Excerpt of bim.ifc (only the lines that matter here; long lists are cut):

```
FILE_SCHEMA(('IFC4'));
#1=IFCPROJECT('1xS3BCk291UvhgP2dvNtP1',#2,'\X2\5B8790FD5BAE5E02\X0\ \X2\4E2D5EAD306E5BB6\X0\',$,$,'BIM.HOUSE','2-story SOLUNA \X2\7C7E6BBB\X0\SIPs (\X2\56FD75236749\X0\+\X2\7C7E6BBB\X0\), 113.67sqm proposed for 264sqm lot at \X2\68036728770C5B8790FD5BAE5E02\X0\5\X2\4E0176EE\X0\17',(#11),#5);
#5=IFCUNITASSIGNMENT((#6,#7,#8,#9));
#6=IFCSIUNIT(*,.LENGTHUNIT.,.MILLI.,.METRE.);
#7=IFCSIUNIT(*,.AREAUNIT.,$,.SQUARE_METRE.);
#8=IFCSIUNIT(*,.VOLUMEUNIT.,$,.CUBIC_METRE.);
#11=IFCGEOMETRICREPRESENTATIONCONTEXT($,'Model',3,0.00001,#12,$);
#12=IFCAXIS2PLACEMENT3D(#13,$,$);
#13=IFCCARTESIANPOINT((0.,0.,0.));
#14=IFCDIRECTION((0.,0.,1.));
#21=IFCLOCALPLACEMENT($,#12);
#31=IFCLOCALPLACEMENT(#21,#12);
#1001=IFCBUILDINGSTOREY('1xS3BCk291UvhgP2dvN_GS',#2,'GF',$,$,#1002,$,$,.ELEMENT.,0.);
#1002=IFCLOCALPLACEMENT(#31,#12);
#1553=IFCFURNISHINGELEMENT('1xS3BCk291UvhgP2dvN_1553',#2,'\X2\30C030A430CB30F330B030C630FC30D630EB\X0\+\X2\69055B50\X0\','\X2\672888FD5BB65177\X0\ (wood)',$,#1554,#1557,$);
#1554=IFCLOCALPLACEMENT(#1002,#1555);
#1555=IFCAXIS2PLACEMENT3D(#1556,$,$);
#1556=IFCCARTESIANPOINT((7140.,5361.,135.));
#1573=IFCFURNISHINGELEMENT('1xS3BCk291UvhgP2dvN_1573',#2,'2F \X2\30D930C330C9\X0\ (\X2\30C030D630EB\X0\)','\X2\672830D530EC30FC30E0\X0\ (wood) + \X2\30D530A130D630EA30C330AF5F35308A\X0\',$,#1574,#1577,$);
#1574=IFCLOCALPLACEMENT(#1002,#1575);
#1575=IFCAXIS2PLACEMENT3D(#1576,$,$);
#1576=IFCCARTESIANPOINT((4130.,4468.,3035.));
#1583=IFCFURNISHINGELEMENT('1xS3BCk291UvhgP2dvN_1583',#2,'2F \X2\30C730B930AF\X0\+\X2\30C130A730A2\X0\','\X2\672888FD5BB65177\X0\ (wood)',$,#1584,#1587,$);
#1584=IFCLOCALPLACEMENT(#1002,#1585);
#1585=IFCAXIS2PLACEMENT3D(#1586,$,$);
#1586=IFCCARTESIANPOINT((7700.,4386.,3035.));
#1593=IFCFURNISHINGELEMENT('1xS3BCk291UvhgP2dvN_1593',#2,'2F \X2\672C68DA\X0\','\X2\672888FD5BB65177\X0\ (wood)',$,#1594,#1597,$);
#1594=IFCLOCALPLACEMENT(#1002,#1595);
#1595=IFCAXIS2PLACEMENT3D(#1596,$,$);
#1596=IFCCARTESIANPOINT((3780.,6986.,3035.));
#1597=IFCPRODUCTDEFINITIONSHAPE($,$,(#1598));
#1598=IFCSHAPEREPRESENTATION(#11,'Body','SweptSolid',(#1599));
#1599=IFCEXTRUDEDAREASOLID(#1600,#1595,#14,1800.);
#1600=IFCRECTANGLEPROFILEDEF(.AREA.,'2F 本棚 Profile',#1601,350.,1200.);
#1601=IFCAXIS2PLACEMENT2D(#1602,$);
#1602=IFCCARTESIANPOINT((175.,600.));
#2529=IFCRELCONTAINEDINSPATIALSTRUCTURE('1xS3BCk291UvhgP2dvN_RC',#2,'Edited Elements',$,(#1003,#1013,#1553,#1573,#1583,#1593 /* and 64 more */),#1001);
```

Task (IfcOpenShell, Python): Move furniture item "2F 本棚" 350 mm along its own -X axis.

```python
import ifcopenshell
import ifcopenshell.api.geometry
import ifcopenshell.util.placement

model = ifcopenshell.open("bim.ifc")

item = model.by_id(1593)
matrix = ifcopenshell.util.placement.get_local_placement(item.ObjectPlacement)
matrix[:3, 3] -= matrix[:3, 0] * 350.0
ifcopenshell.api.geometry.edit_object_placement(model, product=item, matrix=matrix, is_si=False)

print(ifcopenshell.util.placement.get_local_placement(item.ObjectPlacement).round(3) + 0.0)

model.write("bim_updated.ifc")
```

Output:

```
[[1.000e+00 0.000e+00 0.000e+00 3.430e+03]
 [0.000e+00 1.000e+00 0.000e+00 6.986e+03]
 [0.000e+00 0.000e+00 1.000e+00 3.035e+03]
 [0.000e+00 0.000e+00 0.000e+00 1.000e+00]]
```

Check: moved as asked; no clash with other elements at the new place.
